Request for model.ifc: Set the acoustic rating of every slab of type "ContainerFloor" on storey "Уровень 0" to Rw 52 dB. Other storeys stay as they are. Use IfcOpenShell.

First a look at what the model holds.

```python
import ifcopenshell
import ifcopenshell.util.element

model = ifcopenshell.open("model.ifc")
print(model.schema)
storey = next(s for s in model.by_type("IfcBuildingStorey") if s.Name == "Уровень 0")
slabs = [e for e in ifcopenshell.util.element.get_decomposition(storey) if e.is_a("IfcSlab")]
seen = {}
for e in slabs:
    element_type = ifcopenshell.util.element.get_type(e)
    key = (element_type.Name if element_type != e and element_type else None, ifcopenshell.util.element.get_pset(e, "Pset_SlabCommon", "AcousticRating"))
    seen[key] = seen.get(key, 0) + 1
for (name, value), count in sorted(seen.items(), key=str):
    print(count, "x", name, "|", value)
```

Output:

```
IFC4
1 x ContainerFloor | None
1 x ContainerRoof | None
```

```python
import ifcopenshell
import ifcopenshell.api.pset
import ifcopenshell.util.element

model = ifcopenshell.open("model.ifc")

storey = next(s for s in model.by_type("IfcBuildingStorey") if s.Name == "Уровень 0")
slabs = [e for e in ifcopenshell.util.element.get_decomposition(storey) if e.is_a("IfcSlab")]

count = 0
for e in slabs:
    element_type = ifcopenshell.util.element.get_type(e)
    if element_type in (None, e) or element_type.Name != "ContainerFloor":
        continue
    # add_pset returns the element's existing set when there is one.
    pset = ifcopenshell.api.pset.add_pset(model, product=e, name="Pset_SlabCommon")
    ifcopenshell.api.pset.edit_pset(model, pset=pset, properties={"AcousticRating": "Rw 52 dB"})
    count += 1

print(count, "slabs updated")

model.write("model_rev.ifc")
```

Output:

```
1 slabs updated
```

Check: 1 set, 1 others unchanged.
